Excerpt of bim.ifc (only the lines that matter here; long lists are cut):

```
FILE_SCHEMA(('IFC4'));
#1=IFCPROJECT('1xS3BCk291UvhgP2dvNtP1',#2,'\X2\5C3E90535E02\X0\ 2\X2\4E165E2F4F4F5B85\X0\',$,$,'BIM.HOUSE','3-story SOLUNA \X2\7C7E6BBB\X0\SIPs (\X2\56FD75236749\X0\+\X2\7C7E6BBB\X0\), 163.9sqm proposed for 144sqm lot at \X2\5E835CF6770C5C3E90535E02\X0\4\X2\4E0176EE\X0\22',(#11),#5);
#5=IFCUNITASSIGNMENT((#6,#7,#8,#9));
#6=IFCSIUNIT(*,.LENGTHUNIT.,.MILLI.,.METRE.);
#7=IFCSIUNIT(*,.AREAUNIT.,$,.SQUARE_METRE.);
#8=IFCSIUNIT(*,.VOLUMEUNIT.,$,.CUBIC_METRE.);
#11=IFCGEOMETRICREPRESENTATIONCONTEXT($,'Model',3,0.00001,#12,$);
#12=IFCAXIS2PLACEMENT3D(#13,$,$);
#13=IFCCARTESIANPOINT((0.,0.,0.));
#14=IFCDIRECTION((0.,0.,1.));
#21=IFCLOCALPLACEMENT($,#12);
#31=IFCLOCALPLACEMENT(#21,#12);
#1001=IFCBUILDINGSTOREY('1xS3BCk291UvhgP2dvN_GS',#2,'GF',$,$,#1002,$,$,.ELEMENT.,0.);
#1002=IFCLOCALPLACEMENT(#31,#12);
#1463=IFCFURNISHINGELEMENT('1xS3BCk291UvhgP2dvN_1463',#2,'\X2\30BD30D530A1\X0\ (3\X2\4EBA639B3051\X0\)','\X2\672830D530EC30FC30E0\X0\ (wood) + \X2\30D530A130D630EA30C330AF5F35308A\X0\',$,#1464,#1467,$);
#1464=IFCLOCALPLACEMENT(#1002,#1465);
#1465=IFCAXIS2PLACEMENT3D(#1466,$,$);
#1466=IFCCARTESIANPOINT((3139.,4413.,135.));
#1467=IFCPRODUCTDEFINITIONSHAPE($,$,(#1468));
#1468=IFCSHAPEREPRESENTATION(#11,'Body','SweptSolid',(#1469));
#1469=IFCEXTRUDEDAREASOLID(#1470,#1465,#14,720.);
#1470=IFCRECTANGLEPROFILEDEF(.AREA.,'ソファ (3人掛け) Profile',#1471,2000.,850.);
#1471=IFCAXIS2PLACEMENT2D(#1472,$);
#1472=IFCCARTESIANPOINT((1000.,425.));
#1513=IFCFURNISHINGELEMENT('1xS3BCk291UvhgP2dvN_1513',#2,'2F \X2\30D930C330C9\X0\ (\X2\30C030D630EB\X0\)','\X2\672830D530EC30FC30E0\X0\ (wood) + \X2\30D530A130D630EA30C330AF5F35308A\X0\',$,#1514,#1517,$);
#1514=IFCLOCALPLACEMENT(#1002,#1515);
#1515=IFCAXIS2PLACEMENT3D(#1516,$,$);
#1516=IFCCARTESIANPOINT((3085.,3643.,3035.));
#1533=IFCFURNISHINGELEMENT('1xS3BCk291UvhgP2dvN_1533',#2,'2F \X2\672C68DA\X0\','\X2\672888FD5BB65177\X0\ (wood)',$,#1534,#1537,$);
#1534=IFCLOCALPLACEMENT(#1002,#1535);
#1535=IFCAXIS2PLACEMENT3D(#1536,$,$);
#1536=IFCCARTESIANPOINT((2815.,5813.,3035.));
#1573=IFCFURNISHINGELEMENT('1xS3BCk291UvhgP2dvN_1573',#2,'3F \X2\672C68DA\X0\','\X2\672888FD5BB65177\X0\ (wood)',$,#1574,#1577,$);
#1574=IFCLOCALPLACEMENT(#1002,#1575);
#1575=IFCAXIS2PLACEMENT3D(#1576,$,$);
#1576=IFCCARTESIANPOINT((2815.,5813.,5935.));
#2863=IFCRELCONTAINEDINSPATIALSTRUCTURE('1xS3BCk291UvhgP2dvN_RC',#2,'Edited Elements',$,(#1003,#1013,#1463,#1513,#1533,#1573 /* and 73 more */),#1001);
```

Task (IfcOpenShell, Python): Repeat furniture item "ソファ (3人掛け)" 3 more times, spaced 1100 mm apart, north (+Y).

```python
import numpy as np
import ifcopenshell
import ifcopenshell.api.geometry
import ifcopenshell.api.root
import ifcopenshell.util.element
import ifcopenshell.util.placement

model = ifcopenshell.open("bim.ifc")


def reuse_history(source, copy):
    """copy_class also copies each property set's owner history, people and application; keep the originals."""
    for rel in copy.IsDefinedBy:
        if rel.is_a("IfcRelDefinesByProperties") and (history := rel.RelatingPropertyDefinition.OwnerHistory):
            rel.RelatingPropertyDefinition.OwnerHistory = source.OwnerHistory
            ifcopenshell.util.element.remove_deep2(model, history)


source = model.by_guid("1xS3BCk291UvhgP2dvN_1463")
base = ifcopenshell.util.placement.get_local_placement(source.ObjectPlacement)
step = np.array([0.0, 1.0, 0.0]) * 1100.0

for i in range(1, 4):
    copy = ifcopenshell.api.root.copy_class(model, product=source)
    copy.Representation = ifcopenshell.util.element.copy_deep(
        model, source.Representation, exclude=["IfcGeometricRepresentationContext", "IfcRepresentationMap"]
    )
    reuse_history(source, copy)
    matrix = base.copy()
    matrix[:3, 3] += i * step
    print("added at", matrix[:3, 3].round(3) + 0.0)
    ifcopenshell.api.geometry.edit_object_placement(model, product=copy, matrix=matrix, is_si=False)

model.write("bim-out.ifc")
```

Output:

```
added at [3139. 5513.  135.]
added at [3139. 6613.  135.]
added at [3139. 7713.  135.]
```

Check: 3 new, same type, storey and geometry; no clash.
